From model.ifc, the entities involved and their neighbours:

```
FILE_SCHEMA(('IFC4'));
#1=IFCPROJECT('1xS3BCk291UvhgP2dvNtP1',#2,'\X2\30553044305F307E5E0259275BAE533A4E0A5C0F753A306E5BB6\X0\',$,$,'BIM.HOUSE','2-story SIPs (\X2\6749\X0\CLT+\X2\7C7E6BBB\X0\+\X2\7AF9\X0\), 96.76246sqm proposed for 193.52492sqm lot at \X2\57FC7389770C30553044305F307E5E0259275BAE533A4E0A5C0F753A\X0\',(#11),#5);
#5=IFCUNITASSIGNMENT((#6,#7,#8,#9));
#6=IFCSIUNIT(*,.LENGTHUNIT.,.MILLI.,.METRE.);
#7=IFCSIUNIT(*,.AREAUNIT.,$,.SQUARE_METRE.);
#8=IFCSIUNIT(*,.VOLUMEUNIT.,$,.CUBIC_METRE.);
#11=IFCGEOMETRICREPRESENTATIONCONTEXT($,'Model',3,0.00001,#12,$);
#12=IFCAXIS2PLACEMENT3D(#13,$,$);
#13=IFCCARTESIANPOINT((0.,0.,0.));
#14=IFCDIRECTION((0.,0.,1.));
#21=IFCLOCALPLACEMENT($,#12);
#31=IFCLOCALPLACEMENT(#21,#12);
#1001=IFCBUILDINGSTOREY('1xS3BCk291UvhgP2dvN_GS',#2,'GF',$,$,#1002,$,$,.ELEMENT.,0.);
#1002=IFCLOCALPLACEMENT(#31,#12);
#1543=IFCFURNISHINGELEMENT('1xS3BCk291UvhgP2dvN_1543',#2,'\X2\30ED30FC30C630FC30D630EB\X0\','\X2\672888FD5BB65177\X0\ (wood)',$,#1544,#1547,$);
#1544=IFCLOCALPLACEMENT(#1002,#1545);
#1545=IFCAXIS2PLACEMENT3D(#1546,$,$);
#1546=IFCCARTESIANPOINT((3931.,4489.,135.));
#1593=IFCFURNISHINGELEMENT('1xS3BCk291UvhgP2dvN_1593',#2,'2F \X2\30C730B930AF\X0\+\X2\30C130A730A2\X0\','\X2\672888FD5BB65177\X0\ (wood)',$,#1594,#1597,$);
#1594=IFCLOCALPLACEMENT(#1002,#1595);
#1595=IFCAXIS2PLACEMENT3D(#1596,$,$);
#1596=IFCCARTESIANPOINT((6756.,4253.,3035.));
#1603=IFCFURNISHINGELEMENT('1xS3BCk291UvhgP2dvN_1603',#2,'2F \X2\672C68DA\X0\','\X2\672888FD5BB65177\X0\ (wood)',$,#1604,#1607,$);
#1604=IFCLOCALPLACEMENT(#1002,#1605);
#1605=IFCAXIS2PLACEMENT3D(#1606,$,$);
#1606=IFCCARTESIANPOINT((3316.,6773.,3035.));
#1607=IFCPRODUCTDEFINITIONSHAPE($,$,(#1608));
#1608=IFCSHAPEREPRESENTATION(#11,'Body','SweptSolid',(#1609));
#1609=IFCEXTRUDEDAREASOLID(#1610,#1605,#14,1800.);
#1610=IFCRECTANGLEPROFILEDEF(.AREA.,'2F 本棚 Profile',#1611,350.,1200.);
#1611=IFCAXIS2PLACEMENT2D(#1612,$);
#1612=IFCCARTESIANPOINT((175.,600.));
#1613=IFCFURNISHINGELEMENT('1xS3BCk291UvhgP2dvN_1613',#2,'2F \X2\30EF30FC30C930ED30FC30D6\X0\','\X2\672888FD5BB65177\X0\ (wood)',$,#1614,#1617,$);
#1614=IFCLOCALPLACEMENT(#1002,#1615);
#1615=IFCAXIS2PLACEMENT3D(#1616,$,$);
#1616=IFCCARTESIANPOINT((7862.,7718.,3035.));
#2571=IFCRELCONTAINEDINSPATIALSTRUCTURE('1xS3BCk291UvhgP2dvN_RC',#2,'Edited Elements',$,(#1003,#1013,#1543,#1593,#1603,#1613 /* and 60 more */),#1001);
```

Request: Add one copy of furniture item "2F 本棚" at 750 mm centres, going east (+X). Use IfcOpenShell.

```python
import numpy as np
import ifcopenshell
import ifcopenshell.api.geometry
import ifcopenshell.api.root
import ifcopenshell.util.element
import ifcopenshell.util.placement

model = ifcopenshell.open("model.ifc")


def reuse_history(source, copy):
    """copy_class also copies each property set's owner history, people and application; keep the originals."""
    for rel in copy.IsDefinedBy:
        if rel.is_a("IfcRelDefinesByProperties") and (history := rel.RelatingPropertyDefinition.OwnerHistory):
            rel.RelatingPropertyDefinition.OwnerHistory = source.OwnerHistory
            ifcopenshell.util.element.remove_deep2(model, history)


source = model.by_guid("1xS3BCk291UvhgP2dvN_1603")
base = ifcopenshell.util.placement.get_local_placement(source.ObjectPlacement)
step = np.array([1.0, 0.0, 0.0]) * 750.0

for i in range(1, 2):
    copy = ifcopenshell.api.root.copy_class(model, product=source)
    copy.Representation = ifcopenshell.util.element.copy_deep(
        model, source.Representation, exclude=["IfcGeometricRepresentationContext", "IfcRepresentationMap"]
    )
    reuse_history(source, copy)
    matrix = base.copy()
    matrix[:3, 3] += i * step
    print("added at", matrix[:3, 3].round(3) + 0.0)
    ifcopenshell.api.geometry.edit_object_placement(model, product=copy, matrix=matrix, is_si=False)

model.write("model_rev.ifc")
```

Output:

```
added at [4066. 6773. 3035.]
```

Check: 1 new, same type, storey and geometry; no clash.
